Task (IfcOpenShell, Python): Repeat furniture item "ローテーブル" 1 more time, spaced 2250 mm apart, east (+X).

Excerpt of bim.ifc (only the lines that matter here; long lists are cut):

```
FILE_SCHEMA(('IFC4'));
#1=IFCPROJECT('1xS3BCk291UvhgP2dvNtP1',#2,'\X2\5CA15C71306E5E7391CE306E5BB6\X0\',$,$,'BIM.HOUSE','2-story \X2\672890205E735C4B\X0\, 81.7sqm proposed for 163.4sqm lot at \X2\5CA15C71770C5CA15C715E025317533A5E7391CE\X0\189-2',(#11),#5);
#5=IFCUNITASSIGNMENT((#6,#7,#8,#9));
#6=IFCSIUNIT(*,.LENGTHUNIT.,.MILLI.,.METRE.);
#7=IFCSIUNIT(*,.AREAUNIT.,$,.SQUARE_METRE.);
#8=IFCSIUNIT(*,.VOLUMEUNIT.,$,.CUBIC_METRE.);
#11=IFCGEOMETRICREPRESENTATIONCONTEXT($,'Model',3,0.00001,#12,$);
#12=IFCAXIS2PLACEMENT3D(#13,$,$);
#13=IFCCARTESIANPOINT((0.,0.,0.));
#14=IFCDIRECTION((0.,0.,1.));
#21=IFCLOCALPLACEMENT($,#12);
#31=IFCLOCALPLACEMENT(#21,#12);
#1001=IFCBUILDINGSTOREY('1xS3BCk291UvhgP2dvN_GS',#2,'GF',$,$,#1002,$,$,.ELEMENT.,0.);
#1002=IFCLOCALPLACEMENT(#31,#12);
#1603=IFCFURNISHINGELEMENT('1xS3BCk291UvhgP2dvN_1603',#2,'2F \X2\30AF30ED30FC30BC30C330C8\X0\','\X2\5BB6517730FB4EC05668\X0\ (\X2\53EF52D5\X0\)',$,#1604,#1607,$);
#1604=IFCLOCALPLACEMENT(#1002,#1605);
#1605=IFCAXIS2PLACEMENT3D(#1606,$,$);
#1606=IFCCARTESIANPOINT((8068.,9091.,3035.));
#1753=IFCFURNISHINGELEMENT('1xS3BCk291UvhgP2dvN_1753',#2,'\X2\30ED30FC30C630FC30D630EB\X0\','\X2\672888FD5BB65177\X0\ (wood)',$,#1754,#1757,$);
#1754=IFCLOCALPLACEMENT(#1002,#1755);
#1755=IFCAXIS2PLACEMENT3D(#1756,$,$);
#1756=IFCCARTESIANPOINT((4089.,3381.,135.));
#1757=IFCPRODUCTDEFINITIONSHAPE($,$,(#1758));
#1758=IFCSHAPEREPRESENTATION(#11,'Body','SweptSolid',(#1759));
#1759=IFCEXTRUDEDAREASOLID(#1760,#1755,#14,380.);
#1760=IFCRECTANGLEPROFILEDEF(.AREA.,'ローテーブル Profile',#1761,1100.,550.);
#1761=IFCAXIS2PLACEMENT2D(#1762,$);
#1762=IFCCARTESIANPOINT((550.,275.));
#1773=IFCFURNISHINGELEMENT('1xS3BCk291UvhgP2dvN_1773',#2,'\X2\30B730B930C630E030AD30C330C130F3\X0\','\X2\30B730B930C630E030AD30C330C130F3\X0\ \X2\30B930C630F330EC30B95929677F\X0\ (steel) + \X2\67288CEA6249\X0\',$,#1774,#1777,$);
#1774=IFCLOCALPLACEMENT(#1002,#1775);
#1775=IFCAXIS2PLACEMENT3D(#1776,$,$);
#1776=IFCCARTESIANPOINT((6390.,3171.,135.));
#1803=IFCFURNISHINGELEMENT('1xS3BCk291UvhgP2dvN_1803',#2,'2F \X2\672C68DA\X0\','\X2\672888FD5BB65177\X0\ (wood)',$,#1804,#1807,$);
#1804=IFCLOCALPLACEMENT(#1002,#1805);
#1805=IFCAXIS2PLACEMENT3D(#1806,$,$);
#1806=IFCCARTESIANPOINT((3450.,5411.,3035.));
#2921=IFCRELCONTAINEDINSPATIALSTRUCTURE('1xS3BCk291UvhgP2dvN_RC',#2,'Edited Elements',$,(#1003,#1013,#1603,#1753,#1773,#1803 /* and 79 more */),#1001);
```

```python
import numpy as np
import ifcopenshell
import ifcopenshell.api.geometry
import ifcopenshell.api.root
import ifcopenshell.util.element
import ifcopenshell.util.placement

model = ifcopenshell.open("bim.ifc")


def reuse_history(source, copy):
    """copy_class also copies each property set's owner history, people and application; keep the originals."""
    for rel in copy.IsDefinedBy:
        if rel.is_a("IfcRelDefinesByProperties") and (history := rel.RelatingPropertyDefinition.OwnerHistory):
            rel.RelatingPropertyDefinition.OwnerHistory = source.OwnerHistory
            ifcopenshell.util.element.remove_deep2(model, history)


source = model.by_guid("1xS3BCk291UvhgP2dvN_1753")
base = ifcopenshell.util.placement.get_local_placement(source.ObjectPlacement)
step = np.array([1.0, 0.0, 0.0]) * 2250.0

for i in range(1, 2):
    copy = ifcopenshell.api.root.copy_class(model, product=source)
    copy.Representation = ifcopenshell.util.element.copy_deep(
        model, source.Representation, exclude=["IfcGeometricRepresentationContext", "IfcRepresentationMap"]
    )
    reuse_history(source, copy)
    matrix = base.copy()
    matrix[:3, 3] += i * step
    print("added at", matrix[:3, 3].round(3) + 0.0)
    ifcopenshell.api.geometry.edit_object_placement(model, product=copy, matrix=matrix, is_si=False)

model.write("bim_v2.ifc")
```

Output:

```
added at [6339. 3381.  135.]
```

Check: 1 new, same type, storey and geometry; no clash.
